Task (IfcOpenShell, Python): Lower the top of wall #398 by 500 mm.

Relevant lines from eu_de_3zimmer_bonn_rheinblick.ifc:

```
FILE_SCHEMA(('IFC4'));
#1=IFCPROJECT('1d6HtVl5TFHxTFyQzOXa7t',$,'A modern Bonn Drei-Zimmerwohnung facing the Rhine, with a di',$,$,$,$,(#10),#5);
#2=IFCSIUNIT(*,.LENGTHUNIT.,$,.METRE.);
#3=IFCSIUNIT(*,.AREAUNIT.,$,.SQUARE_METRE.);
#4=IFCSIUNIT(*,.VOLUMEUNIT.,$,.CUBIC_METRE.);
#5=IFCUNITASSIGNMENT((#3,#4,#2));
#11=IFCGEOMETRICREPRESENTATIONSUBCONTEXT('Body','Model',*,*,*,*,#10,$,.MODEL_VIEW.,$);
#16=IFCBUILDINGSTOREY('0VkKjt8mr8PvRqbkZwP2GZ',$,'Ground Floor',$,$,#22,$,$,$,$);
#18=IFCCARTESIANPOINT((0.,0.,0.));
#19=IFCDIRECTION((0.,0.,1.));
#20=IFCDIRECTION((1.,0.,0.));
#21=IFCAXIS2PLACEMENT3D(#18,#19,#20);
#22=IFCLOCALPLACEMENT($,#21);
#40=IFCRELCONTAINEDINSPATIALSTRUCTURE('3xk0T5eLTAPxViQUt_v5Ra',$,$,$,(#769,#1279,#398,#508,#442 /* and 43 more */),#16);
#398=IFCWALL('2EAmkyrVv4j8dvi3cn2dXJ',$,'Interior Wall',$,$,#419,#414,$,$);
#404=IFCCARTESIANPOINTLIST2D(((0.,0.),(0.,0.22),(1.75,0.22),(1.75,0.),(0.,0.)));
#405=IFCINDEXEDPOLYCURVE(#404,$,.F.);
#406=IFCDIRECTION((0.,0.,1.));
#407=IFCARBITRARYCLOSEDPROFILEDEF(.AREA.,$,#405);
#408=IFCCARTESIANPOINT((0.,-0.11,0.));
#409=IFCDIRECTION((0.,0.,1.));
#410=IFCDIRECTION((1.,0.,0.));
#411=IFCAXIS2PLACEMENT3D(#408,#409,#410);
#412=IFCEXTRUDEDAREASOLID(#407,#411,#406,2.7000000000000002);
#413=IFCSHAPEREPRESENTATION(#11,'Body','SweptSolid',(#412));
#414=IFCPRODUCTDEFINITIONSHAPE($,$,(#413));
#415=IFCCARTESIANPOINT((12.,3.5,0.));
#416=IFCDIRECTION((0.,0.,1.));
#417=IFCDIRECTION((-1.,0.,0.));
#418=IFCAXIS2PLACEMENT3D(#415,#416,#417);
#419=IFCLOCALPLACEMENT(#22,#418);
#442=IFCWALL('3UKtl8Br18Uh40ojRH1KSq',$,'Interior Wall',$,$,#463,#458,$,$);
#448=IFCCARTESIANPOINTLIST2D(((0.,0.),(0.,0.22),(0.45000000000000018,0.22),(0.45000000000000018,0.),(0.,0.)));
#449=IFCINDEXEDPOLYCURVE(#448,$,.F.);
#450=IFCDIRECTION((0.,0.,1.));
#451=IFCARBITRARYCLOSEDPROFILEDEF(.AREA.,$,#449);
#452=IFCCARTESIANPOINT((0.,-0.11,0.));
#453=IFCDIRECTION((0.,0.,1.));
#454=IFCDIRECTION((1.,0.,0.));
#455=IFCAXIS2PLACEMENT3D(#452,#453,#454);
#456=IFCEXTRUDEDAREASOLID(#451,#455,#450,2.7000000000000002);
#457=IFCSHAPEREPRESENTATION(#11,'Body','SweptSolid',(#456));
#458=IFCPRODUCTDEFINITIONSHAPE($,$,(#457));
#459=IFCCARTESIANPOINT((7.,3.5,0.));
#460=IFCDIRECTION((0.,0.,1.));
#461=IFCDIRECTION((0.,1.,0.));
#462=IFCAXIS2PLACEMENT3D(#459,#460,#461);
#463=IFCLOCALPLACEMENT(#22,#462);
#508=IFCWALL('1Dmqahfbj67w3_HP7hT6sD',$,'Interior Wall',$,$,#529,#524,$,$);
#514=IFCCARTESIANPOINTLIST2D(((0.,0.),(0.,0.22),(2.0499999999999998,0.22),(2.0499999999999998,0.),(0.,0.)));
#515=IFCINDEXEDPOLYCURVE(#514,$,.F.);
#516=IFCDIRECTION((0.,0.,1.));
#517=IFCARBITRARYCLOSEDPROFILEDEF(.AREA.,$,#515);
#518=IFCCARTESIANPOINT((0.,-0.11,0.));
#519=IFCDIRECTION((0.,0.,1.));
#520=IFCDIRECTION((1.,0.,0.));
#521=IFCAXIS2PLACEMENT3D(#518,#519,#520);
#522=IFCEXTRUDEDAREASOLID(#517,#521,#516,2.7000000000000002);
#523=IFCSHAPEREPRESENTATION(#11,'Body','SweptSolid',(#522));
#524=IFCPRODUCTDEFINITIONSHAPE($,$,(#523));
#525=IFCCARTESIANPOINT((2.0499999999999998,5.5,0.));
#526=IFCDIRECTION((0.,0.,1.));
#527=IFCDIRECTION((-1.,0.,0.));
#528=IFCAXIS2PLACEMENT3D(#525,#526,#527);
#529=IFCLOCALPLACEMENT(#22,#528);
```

```python
import ifcopenshell
import ifcopenshell.geom
import ifcopenshell.util.representation
import ifcopenshell.util.shape
import ifcopenshell.util.unit

model = ifcopenshell.open("eu_de_3zimmer_bonn_rheinblick.ifc")
unit_scale = ifcopenshell.util.unit.calculate_unit_scale(model)
settings = ifcopenshell.geom.settings()


def volume(element):
    """Net volume in cubic metres, openings subtracted."""
    shape = ifcopenshell.geom.create_shape(settings, element)
    return ifcopenshell.util.shape.get_volume(shape.geometry)


wall = model.by_id(398)
before = volume(wall)

body = ifcopenshell.util.representation.get_representation(wall, "Model", "Body")
solid = body.Items[0]
old_height = solid.Depth
solid.Depth -= 0.5 / unit_scale
after = volume(wall)

print(f"height {old_height:g} -> {solid.Depth:g}, volume {before:.3f} -> {after:.3f} m3")

model.write("eu_de_3zimmer_bonn_rheinblick_updated.ifc")
```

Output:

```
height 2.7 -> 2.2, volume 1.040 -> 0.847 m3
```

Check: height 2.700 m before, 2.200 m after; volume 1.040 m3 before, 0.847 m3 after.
